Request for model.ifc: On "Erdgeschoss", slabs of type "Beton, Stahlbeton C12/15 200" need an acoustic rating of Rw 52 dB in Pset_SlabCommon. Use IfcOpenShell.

First a look at what the model holds.

```python
import ifcopenshell
import ifcopenshell.util.element

model = ifcopenshell.open("model.ifc")
print(model.schema)
storey = next(s for s in model.by_type("IfcBuildingStorey") if s.Name == "Erdgeschoss")
slabs = [e for e in ifcopenshell.util.element.get_decomposition(storey) if e.is_a("IfcSlab")]
seen = {}
for e in slabs:
    element_type = ifcopenshell.util.element.get_type(e)
    key = (element_type.Name if element_type != e and element_type else None, ifcopenshell.util.element.get_pset(e, "Pset_SlabCommon", "AcousticRating"))
    seen[key] = seen.get(key, 0) + 1
for (name, value), count in sorted(seen.items(), key=str):
    print(count, "x", name, "|", value)
```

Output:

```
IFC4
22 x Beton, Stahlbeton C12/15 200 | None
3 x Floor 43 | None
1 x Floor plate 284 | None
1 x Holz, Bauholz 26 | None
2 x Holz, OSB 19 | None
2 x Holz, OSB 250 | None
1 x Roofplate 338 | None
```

```python
import ifcopenshell
import ifcopenshell.api.pset
import ifcopenshell.util.element

model = ifcopenshell.open("model.ifc")

storey = next(s for s in model.by_type("IfcBuildingStorey") if s.Name == "Erdgeschoss")
slabs = [e for e in ifcopenshell.util.element.get_decomposition(storey) if e.is_a("IfcSlab")]

count = 0
for e in slabs:
    element_type = ifcopenshell.util.element.get_type(e)
    if element_type in (None, e) or element_type.Name != "Beton, Stahlbeton C12/15 200":
        continue
    # add_pset returns the element's existing set when there is one.
    pset = ifcopenshell.api.pset.add_pset(model, product=e, name="Pset_SlabCommon")
    ifcopenshell.api.pset.edit_pset(model, pset=pset, properties={"AcousticRating": "Rw 52 dB"})
    count += 1

print(count, "slabs updated")

model.write("model_updated.ifc")
```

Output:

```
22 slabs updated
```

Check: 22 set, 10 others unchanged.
